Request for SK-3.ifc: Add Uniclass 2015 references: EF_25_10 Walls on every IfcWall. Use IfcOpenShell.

First a look at what the model holds.

```python
import ifcopenshell

model = ifcopenshell.open("SK-3.ifc")
print(model.schema)
print("classifications:", [c.Name for c in model.by_type("IfcClassification")])
for ifc_class in ("IfcDoor", "IfcRoof", "IfcStair", "IfcWall", "IfcWindow"):
    print(ifc_class, len(model.by_type(ifc_class)))
```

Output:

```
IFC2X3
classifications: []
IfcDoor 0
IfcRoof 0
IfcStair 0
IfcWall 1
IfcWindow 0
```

```python
import ifcopenshell
import ifcopenshell.api.classification

model = ifcopenshell.open("SK-3.ifc")

# IFC2X3 requires Source and Edition and has no link from the project to the system.
system = model.create_entity("IfcClassification", Source="NBS", Edition="2015", Name="Uniclass 2015")

codes = {
    "IfcWall": ("EF_25_10", "Walls"),
}
for ifc_class, (code, name) in codes.items():
    products = model.by_type(ifc_class)
    ifcopenshell.api.classification.add_reference(
        model, products=products, classification=system, identification=code, name=name
    )
    print(code, len(products))

model.write("SK-3_v2.ifc")
```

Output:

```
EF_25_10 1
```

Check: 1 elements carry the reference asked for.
